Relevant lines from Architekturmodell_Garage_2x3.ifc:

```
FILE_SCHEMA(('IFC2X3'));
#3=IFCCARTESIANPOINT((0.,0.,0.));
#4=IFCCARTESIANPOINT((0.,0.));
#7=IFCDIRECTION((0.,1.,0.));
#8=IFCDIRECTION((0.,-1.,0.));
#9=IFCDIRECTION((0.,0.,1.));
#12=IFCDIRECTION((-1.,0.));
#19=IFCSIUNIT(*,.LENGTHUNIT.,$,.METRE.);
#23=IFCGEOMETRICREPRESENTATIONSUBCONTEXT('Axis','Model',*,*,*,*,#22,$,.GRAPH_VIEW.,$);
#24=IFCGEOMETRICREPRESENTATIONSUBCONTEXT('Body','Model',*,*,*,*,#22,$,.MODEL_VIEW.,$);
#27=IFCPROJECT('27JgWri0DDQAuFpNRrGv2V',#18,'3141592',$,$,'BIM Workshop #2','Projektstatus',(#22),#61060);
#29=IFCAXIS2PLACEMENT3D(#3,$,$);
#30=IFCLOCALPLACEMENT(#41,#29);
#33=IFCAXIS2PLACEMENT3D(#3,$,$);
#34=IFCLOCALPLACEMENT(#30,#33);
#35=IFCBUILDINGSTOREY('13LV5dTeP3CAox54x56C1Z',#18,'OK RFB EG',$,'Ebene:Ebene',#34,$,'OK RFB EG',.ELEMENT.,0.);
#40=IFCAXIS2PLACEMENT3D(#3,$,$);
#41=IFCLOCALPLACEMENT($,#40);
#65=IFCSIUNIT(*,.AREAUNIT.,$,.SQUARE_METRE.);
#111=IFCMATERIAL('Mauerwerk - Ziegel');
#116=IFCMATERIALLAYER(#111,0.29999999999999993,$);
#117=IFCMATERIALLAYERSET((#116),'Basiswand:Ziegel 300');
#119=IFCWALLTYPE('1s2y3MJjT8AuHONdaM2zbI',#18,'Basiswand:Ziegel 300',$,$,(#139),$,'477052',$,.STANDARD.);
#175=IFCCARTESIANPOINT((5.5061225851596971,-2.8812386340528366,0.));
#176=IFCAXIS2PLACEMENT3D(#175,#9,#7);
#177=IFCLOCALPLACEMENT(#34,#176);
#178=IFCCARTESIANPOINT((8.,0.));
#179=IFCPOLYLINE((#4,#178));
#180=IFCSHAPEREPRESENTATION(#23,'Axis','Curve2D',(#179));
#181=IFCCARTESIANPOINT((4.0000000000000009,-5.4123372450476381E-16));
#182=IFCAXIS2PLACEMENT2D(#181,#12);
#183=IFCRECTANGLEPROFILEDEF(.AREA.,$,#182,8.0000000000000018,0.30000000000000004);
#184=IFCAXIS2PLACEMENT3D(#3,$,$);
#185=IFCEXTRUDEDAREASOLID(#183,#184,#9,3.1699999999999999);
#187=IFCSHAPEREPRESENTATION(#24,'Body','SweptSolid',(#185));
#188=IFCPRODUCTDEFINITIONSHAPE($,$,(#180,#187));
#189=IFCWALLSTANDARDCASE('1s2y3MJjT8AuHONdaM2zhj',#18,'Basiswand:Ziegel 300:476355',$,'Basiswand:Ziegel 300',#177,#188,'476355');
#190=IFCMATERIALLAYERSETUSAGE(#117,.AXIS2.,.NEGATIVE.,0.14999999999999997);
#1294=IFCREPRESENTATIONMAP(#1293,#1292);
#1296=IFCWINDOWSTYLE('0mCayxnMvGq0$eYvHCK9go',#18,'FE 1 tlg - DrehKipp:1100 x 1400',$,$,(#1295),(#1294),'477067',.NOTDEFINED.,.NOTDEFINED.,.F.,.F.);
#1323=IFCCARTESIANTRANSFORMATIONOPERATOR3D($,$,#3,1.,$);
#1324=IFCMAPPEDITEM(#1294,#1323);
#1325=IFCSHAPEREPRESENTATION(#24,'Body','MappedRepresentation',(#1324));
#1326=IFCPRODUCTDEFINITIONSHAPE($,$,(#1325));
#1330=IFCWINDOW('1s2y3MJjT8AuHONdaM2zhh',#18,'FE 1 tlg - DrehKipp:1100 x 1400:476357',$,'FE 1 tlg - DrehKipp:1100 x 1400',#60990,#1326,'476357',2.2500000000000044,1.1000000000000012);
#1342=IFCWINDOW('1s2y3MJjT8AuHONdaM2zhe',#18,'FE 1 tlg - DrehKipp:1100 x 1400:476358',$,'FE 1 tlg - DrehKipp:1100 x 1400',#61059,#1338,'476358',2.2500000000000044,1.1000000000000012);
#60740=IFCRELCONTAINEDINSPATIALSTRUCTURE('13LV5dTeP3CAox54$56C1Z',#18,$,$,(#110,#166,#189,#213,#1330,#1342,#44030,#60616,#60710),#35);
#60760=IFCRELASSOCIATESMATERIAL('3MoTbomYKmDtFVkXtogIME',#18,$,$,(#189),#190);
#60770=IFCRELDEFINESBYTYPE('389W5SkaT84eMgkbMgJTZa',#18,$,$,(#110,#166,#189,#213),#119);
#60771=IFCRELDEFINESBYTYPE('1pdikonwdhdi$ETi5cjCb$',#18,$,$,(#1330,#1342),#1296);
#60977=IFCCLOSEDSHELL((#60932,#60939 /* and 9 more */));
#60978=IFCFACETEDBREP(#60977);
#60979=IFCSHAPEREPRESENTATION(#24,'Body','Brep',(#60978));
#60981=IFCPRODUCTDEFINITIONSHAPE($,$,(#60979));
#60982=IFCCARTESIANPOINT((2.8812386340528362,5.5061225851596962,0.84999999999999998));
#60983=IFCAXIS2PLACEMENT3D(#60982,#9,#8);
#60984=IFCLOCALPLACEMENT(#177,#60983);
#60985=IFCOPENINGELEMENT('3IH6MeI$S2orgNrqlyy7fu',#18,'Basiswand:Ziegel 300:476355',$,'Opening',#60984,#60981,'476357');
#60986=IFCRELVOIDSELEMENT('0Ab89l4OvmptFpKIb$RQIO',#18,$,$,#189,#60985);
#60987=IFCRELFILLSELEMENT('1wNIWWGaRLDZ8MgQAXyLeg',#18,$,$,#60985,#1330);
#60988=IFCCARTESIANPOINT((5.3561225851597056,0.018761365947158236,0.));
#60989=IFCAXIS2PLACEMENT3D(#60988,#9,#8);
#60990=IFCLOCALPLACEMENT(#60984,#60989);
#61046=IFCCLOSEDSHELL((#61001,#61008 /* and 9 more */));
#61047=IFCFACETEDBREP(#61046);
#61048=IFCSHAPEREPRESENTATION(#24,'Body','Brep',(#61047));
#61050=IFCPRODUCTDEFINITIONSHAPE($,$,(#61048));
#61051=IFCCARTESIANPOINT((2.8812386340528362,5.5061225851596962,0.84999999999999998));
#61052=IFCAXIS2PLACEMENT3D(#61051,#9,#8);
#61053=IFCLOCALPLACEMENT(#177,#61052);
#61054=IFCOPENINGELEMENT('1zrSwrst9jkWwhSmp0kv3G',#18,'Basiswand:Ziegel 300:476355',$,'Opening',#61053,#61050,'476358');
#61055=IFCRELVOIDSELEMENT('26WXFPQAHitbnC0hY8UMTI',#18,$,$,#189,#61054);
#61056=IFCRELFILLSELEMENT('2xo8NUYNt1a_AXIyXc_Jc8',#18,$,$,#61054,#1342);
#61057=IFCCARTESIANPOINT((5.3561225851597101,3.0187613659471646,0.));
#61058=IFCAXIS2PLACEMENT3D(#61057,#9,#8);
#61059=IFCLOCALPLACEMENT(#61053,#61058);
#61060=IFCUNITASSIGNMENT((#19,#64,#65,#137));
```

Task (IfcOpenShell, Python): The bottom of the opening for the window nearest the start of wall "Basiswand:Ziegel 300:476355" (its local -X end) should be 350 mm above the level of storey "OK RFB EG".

```python
import numpy as np
import ifcopenshell
import ifcopenshell.api.geometry
import ifcopenshell.geom
import ifcopenshell.util.element
import ifcopenshell.util.placement
import ifcopenshell.util.shape
import ifcopenshell.util.unit

model = ifcopenshell.open("Architekturmodell_Garage_2x3.ifc")
unit_scale = ifcopenshell.util.unit.calculate_unit_scale(model)

window = model.by_id(1330)
opening = window.FillsVoids[0].RelatingOpeningElement
storey = ifcopenshell.util.element.get_container(window, ifc_class="IfcBuildingStorey")
level = ifcopenshell.util.placement.get_local_placement(storey.ObjectPlacement)[2, 3]

# The opening's origin need not be at the sill, so measure its lowest point.
shape = ifcopenshell.geom.create_shape(ifcopenshell.geom.settings(), opening)
bottom = ifcopenshell.util.shape.get_shape_bottom_elevation(shape, shape.geometry) / unit_scale
dz = level + 0.35 - bottom

shift = np.array([0.0, 0.0, dz])
# The window is placed relative to its opening, so it follows when the opening moves.
matrix = ifcopenshell.util.placement.get_local_placement(opening.ObjectPlacement)
matrix[:3, 3] += shift
ifcopenshell.api.geometry.edit_object_placement(
    model, product=opening, matrix=matrix, is_si=False, should_transform_children=True
)

print(f"moved by {dz * unit_scale:+.3f} m")

model.write("Architekturmodell_Garage_2x3_v2.ifc")
```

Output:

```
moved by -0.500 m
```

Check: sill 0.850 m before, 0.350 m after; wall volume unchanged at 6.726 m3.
